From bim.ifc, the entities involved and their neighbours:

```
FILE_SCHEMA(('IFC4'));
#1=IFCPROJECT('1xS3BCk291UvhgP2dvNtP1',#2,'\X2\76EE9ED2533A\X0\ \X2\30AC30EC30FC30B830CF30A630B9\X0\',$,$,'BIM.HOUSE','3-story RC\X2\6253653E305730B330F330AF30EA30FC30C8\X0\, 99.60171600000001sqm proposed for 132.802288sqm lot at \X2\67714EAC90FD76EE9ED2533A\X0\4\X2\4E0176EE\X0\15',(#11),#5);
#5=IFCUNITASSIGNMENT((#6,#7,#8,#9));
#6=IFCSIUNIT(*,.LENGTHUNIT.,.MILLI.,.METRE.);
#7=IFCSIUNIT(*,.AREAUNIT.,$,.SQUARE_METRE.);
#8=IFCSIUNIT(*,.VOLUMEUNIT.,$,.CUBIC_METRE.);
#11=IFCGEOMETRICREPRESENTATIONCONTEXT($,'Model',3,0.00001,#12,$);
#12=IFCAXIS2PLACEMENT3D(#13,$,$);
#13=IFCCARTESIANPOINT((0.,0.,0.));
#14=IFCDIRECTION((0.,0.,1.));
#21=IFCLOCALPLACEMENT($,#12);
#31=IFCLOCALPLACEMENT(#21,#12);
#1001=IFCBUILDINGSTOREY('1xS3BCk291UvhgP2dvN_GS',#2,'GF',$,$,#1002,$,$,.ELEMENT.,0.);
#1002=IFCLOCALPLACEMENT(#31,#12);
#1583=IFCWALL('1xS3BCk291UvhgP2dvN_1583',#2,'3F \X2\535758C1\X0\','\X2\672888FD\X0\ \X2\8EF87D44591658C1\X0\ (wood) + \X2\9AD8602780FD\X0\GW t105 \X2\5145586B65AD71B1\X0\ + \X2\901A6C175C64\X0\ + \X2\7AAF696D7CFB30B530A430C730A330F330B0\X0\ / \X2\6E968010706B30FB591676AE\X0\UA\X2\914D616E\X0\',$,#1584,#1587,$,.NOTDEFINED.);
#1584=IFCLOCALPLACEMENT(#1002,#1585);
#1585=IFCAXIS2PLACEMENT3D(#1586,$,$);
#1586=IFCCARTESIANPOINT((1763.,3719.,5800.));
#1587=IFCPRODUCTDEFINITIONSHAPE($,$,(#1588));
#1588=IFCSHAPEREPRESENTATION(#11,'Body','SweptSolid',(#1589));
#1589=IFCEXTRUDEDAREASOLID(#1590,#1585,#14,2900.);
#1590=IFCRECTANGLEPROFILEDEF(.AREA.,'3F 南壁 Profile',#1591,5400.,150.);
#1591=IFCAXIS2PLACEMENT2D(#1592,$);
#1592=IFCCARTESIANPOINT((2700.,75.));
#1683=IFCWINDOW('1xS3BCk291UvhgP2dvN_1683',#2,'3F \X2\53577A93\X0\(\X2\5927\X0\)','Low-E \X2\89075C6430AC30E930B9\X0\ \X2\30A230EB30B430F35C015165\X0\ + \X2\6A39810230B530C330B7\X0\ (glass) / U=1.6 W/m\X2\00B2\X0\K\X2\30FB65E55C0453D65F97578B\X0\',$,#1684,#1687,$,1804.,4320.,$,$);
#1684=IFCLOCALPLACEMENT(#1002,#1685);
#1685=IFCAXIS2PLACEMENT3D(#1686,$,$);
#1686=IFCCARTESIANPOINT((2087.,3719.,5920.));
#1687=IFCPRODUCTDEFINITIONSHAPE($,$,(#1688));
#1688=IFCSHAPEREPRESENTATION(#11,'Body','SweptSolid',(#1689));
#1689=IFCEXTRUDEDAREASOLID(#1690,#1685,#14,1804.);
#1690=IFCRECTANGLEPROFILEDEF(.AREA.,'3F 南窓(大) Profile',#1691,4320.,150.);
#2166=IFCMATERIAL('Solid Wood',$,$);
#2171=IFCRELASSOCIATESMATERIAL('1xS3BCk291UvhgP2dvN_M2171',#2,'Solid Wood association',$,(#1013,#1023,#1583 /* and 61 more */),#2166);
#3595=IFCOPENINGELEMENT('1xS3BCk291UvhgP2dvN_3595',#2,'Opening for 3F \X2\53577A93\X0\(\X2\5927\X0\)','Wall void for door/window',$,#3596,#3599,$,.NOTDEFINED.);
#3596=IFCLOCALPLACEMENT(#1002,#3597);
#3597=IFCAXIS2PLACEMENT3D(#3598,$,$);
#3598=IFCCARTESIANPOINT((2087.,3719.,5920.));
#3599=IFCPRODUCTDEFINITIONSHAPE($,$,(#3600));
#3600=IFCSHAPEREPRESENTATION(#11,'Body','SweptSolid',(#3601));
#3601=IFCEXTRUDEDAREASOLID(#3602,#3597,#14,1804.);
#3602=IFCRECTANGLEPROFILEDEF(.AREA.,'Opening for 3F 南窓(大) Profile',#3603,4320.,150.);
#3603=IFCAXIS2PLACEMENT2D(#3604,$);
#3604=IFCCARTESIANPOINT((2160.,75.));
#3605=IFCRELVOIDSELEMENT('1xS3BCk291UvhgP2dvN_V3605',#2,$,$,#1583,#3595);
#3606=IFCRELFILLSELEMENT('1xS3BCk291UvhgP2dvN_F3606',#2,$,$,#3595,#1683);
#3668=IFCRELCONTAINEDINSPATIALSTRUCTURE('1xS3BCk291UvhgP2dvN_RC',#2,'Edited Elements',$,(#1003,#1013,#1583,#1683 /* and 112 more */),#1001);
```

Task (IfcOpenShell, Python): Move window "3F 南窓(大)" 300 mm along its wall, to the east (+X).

```python
import ifcopenshell
import ifcopenshell.api.geometry
import ifcopenshell.util.placement
import ifcopenshell.util.unit

model = ifcopenshell.open("bim.ifc")
unit_scale = ifcopenshell.util.unit.calculate_unit_scale(model)

window = model.by_guid("1xS3BCk291UvhgP2dvN_1683")
opening = window.FillsVoids[0].RelatingOpeningElement
wall = opening.VoidsElements[0].RelatingBuildingElement

wall_matrix = ifcopenshell.util.placement.get_local_placement(wall.ObjectPlacement)
shift = wall_matrix[:3, 0] * 0.3 / unit_scale
before = ifcopenshell.util.placement.get_local_placement(window.ObjectPlacement)[:3, 3].copy()

# The window is not placed relative to its opening, so move both.
for product in (opening, window):
    matrix = ifcopenshell.util.placement.get_local_placement(product.ObjectPlacement)
    matrix[:3, 3] += shift
    ifcopenshell.api.geometry.edit_object_placement(model, product=product, matrix=matrix, is_si=False)

after = ifcopenshell.util.placement.get_local_placement(window.ObjectPlacement)[:3, 3]
print("window moved by", (after - before).round(3) + 0.0)

model.write("bim_updated.ifc")
```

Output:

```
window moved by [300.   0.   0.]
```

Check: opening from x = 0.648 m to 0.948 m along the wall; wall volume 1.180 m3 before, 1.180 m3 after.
